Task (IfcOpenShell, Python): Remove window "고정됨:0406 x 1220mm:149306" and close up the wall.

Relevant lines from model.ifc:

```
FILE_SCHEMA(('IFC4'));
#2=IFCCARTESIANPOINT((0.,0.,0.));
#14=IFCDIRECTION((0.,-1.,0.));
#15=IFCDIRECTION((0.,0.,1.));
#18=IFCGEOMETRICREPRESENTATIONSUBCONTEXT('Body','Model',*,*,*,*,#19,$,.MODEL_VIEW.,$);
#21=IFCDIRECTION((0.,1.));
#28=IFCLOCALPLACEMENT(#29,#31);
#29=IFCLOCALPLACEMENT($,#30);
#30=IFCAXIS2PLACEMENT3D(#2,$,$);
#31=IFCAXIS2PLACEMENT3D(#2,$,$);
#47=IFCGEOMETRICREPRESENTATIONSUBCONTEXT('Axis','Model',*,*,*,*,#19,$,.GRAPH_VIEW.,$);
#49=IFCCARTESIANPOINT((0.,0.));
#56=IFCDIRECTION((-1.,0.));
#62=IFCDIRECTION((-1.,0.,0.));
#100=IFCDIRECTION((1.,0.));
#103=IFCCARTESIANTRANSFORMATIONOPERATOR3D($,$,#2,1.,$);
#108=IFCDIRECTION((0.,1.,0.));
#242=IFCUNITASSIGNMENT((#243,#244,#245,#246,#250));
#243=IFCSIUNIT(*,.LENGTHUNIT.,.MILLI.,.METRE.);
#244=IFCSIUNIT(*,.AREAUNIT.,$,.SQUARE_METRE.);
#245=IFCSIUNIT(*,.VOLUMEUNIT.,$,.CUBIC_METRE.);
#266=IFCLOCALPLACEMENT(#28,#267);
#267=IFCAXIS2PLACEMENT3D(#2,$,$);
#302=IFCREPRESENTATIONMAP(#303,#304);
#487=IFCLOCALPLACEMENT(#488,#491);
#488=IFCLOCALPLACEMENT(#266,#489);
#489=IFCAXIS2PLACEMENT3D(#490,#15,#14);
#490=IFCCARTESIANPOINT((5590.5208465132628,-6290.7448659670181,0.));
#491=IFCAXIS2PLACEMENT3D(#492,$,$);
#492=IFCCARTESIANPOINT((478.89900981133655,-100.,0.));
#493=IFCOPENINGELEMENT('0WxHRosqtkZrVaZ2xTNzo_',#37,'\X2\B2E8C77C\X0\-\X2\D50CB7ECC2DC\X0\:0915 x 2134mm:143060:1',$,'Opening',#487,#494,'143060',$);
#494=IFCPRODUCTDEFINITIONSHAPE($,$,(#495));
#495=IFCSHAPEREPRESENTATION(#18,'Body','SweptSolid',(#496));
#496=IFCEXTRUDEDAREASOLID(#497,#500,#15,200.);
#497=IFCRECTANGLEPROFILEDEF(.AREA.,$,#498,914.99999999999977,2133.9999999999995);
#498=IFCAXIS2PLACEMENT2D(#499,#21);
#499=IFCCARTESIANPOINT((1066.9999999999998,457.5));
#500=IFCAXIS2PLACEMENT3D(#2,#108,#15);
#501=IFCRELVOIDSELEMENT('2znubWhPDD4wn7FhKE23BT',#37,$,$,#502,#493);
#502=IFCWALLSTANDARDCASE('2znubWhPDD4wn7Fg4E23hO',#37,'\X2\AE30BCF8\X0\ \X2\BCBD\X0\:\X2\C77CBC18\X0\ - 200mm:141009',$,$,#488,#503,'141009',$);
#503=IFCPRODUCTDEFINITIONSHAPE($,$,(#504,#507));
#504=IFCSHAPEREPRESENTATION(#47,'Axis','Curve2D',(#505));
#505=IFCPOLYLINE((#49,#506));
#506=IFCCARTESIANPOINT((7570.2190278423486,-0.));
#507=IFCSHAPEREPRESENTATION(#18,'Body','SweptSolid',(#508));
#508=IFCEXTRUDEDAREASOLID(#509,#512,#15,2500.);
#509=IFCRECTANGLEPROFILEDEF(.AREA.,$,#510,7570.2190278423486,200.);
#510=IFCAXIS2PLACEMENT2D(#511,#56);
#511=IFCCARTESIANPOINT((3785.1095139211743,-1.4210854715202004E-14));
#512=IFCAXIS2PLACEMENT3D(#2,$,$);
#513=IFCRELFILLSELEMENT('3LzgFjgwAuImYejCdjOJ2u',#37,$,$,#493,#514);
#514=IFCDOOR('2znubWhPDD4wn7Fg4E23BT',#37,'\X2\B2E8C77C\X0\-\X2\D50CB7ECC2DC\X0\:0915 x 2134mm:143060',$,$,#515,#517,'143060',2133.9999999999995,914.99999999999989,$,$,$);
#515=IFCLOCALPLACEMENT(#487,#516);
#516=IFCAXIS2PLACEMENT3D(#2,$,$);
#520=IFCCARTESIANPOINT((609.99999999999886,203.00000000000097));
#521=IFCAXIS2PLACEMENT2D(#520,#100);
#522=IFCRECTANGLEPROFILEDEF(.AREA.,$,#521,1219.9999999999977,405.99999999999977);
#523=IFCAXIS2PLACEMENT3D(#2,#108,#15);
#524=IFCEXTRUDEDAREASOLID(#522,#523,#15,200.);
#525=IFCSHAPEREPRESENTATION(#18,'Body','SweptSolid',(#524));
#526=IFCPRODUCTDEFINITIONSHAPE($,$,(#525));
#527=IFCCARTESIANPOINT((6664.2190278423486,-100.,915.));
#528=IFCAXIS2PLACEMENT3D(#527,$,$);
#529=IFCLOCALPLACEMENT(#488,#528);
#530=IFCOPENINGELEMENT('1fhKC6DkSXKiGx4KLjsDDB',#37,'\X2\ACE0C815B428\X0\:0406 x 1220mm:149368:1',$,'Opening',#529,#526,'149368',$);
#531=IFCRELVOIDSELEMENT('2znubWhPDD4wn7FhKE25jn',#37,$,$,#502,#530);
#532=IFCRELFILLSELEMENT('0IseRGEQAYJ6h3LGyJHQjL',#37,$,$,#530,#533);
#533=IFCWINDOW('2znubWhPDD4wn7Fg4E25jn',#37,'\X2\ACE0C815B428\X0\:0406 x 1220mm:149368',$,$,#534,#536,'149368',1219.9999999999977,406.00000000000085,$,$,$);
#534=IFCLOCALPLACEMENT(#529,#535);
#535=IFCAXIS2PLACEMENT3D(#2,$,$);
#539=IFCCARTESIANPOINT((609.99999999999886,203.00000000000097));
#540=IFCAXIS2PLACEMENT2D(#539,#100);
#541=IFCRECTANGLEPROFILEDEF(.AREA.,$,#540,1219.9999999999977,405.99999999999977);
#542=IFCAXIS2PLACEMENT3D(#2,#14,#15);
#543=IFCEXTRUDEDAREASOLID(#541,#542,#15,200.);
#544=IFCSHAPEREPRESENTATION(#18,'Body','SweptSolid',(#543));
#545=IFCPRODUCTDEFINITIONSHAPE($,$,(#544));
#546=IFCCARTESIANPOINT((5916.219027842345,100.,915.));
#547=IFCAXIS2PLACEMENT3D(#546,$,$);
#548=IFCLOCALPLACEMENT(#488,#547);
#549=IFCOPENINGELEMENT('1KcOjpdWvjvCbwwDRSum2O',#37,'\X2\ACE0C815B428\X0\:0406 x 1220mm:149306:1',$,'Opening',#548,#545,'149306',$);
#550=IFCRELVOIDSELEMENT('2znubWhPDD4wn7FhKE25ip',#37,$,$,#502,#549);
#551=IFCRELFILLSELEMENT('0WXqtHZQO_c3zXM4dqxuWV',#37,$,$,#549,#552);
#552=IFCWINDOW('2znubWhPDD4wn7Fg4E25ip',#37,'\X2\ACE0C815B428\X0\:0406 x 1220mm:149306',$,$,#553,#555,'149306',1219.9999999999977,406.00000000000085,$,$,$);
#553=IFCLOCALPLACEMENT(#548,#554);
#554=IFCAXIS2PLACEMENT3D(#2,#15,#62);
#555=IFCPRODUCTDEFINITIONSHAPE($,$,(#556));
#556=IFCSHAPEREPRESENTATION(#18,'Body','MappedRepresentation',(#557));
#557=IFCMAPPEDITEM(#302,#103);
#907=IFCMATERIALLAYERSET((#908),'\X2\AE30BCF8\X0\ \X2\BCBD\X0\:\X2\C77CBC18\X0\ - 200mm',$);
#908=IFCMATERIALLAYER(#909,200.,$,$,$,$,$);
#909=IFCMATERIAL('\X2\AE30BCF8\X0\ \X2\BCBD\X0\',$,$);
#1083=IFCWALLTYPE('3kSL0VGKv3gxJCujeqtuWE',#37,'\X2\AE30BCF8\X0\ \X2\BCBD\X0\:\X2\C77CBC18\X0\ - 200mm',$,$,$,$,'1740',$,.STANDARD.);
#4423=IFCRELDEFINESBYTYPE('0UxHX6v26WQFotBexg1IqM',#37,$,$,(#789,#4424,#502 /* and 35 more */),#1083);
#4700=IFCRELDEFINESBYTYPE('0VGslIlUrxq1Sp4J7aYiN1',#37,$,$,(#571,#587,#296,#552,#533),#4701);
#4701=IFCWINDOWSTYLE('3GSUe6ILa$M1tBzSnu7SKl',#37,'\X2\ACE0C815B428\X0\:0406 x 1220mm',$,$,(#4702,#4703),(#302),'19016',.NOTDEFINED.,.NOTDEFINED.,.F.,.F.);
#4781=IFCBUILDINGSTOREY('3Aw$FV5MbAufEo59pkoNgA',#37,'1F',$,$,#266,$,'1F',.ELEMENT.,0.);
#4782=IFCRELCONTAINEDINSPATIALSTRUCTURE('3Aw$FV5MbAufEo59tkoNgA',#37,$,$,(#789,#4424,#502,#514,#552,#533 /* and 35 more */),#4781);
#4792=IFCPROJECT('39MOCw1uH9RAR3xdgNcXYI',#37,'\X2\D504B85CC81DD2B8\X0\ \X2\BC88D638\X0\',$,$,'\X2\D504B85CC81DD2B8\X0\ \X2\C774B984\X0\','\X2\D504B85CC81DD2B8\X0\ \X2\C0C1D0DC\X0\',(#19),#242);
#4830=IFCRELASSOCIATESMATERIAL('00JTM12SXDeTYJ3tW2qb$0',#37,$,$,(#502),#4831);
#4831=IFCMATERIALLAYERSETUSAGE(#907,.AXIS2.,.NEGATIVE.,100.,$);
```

```python
import ifcopenshell
import ifcopenshell.api.feature
import ifcopenshell.api.root
import ifcopenshell.geom
import ifcopenshell.util.shape

model = ifcopenshell.open("model.ifc")
settings = ifcopenshell.geom.settings()


def volume(element):
    """Net volume in cubic metres, openings subtracted."""
    shape = ifcopenshell.geom.create_shape(settings, element)
    return ifcopenshell.util.shape.get_volume(shape.geometry)


window = model.by_guid("2znubWhPDD4wn7Fg4E25ip")
opening = window.FillsVoids[0].RelatingOpeningElement
wall = opening.VoidsElements[0].RelatingBuildingElement
before = volume(wall)

ifcopenshell.api.root.remove_product(model, product=window)
ifcopenshell.api.feature.remove_feature(model, feature=opening)

after = volume(wall)

print(f"wall volume {before:.3f} -> {after:.3f} m3")

model.write("model_edited.ifc")
```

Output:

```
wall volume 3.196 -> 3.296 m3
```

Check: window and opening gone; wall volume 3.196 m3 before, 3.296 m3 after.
